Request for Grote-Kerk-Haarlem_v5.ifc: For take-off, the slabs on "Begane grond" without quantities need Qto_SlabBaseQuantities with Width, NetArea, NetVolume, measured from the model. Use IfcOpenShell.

First a look at what the model holds.

```python
import ifcopenshell
import ifcopenshell.util.element
import ifcopenshell.util.unit

model = ifcopenshell.open("Grote-Kerk-Haarlem_v5.ifc")
print(model.schema)
for unit_type in ("LENGTHUNIT", "AREAUNIT", "VOLUMEUNIT"):
    print(unit_type, ifcopenshell.util.unit.calculate_unit_scale(model, unit_type))
storey = next(s for s in model.by_type("IfcBuildingStorey") if s.Name == "Begane grond")
slabs = [e for e in ifcopenshell.util.element.get_decomposition(storey) if e.is_a("IfcSlab")]
for e in sorted(slabs, key=lambda e: e.id()):
    print(e.id(), e.is_a(), e.Name, list(ifcopenshell.util.element.get_psets(e, qtos_only=True)), sep=" | ")
```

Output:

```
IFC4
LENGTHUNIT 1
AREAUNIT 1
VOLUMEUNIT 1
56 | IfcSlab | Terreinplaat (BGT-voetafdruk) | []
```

```python
import ifcopenshell
import ifcopenshell.api.pset
import ifcopenshell.geom
import ifcopenshell.util.element
import ifcopenshell.util.shape
import ifcopenshell.util.unit

model = ifcopenshell.open("Grote-Kerk-Haarlem_v5.ifc")
unit_scale = ifcopenshell.util.unit.calculate_unit_scale(model)
area_scale = ifcopenshell.util.unit.calculate_unit_scale(model, "AREAUNIT")
volume_scale = ifcopenshell.util.unit.calculate_unit_scale(model, "VOLUMEUNIT")
settings = ifcopenshell.geom.settings()

storey = next(s for s in model.by_type("IfcBuildingStorey") if s.Name == "Begane grond")
slabs = [e for e in ifcopenshell.util.element.get_decomposition(storey) if e.is_a("IfcSlab")]

for e in sorted(slabs, key=lambda e: e.id()):
    if ifcopenshell.util.element.get_psets(e, qtos_only=True, should_inherit=False):
        continue
    # Geometry comes back in metres, in the element's own axes.
    shape = ifcopenshell.geom.create_shape(settings, e)
    values = {
        "Width": ifcopenshell.util.shape.get_z(shape.geometry) / unit_scale,
        "NetArea": ifcopenshell.util.shape.get_footprint_area(shape.geometry) / area_scale,
        "NetVolume": ifcopenshell.util.shape.get_volume(shape.geometry) / volume_scale,
    }
    qto = ifcopenshell.api.pset.add_qto(model, product=e, name="Qto_SlabBaseQuantities")
    ifcopenshell.api.pset.edit_qto(model, qto=qto, properties=values)
    print(e.id(), {k: round(v, 3) for k, v in values.items()})

model.write("Grote-Kerk-Haarlem_v5-out.ifc")
```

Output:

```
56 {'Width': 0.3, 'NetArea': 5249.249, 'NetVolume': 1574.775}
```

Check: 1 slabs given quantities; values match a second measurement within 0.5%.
